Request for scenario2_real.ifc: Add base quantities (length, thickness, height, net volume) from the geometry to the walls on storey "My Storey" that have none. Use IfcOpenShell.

First a look at what the model holds.

```python
import ifcopenshell
import ifcopenshell.util.element
import ifcopenshell.util.unit

model = ifcopenshell.open("scenario2_real.ifc")
print(model.schema)
for unit_type in ("LENGTHUNIT", "AREAUNIT", "VOLUMEUNIT"):
    print(unit_type, ifcopenshell.util.unit.calculate_unit_scale(model, unit_type))
storey = next(s for s in model.by_type("IfcBuildingStorey") if s.Name == "My Storey")
walls = [e for e in ifcopenshell.util.element.get_decomposition(storey) if e.is_a("IfcWall")]
for e in sorted(walls, key=lambda e: e.id()):
    print(e.id(), e.is_a(), e.Name, list(ifcopenshell.util.element.get_psets(e, qtos_only=True)), sep=" | ")
```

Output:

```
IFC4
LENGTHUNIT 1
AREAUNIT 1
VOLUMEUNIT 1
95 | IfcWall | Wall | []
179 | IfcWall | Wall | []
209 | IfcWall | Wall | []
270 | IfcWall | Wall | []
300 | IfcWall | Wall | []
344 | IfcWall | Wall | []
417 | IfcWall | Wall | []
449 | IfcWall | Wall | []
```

```python
import ifcopenshell
import ifcopenshell.api.pset
import ifcopenshell.geom
import ifcopenshell.util.element
import ifcopenshell.util.shape
import ifcopenshell.util.unit

model = ifcopenshell.open("scenario2_real.ifc")
unit_scale = ifcopenshell.util.unit.calculate_unit_scale(model)
volume_scale = ifcopenshell.util.unit.calculate_unit_scale(model, "VOLUMEUNIT")
settings = ifcopenshell.geom.settings()

storey = next(s for s in model.by_type("IfcBuildingStorey") if s.Name == "My Storey")
walls = [e for e in ifcopenshell.util.element.get_decomposition(storey) if e.is_a("IfcWall")]

for e in sorted(walls, key=lambda e: e.id()):
    if ifcopenshell.util.element.get_psets(e, qtos_only=True, should_inherit=False):
        continue
    # Geometry comes back in metres, in the element's own axes.
    shape = ifcopenshell.geom.create_shape(settings, e)
    values = {
        "Length": ifcopenshell.util.shape.get_x(shape.geometry) / unit_scale,
        "Width": ifcopenshell.util.shape.get_y(shape.geometry) / unit_scale,
        "Height": ifcopenshell.util.shape.get_z(shape.geometry) / unit_scale,
        "NetVolume": ifcopenshell.util.shape.get_volume(shape.geometry) / volume_scale,
    }
    qto = ifcopenshell.api.pset.add_qto(model, product=e, name="Qto_WallBaseQuantities")
    ifcopenshell.api.pset.edit_qto(model, qto=qto, properties=values)
    print(e.id(), {k: round(v, 3) for k, v in values.items()})

model.write("scenario2_real_edited.ifc")
```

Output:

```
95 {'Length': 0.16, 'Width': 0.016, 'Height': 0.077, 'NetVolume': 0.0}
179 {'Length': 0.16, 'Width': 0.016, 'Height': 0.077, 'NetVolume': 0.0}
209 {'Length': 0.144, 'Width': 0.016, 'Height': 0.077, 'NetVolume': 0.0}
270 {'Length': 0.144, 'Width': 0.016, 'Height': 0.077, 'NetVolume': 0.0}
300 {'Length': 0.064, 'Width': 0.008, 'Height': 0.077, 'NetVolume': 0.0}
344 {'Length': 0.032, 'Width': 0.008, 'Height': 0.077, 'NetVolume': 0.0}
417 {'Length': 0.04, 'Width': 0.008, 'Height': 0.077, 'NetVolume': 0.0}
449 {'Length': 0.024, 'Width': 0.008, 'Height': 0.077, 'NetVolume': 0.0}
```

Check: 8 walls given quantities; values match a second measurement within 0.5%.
